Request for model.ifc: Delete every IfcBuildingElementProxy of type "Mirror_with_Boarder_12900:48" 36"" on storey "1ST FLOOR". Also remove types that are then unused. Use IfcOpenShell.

First a look at what the model holds.

```python
import ifcopenshell
import ifcopenshell.util.element

model = ifcopenshell.open("model.ifc")
print(model.schema)
storey = next(s for s in model.by_type("IfcBuildingStorey") if s.Name == "1ST FLOOR")
proxies = [e for e in ifcopenshell.util.element.get_decomposition(storey) if e.is_a("IfcBuildingElementProxy")]
seen = {}
for e in proxies:
    element_type = ifcopenshell.util.element.get_type(e)
    name = element_type.Name if element_type not in (None, e) else None
    seen[name] = seen.get(name, 0) + 1
for name, count in sorted(seen.items(), key=str):
    print(count, "x", name)
```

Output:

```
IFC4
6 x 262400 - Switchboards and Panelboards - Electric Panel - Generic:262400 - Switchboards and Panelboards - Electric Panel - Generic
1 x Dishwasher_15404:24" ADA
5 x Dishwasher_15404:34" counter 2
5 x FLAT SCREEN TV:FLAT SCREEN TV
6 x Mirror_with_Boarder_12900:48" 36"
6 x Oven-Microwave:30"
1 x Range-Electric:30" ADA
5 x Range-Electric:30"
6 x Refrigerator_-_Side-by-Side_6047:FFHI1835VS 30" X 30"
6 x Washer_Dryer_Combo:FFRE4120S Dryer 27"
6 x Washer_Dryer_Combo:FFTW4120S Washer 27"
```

```python
import ifcopenshell
import ifcopenshell.api.root
import ifcopenshell.util.element

model = ifcopenshell.open("model.ifc")

storey = next(s for s in model.by_type("IfcBuildingStorey") if s.Name == "1ST FLOOR")
proxies = [e for e in ifcopenshell.util.element.get_decomposition(storey) if e.is_a("IfcBuildingElementProxy")]
targets = [e for e in proxies if (t := ifcopenshell.util.element.get_type(e)) not in (None, e) and t.Name == 'Mirror_with_Boarder_12900:48" 36"']
types = {ifcopenshell.util.element.get_type(e) for e in targets} - {None, *targets}

for e in targets:
    ifcopenshell.api.root.remove_product(model, product=e)
print(len(targets), "removed")

unused = [t for t in types if not ifcopenshell.util.element.get_types(t)]
for t in unused:
    ifcopenshell.api.root.remove_product(model, product=t)
print(len(unused), "unused types removed")

model.write("model-out.ifc")
```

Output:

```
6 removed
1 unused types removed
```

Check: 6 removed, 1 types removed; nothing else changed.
